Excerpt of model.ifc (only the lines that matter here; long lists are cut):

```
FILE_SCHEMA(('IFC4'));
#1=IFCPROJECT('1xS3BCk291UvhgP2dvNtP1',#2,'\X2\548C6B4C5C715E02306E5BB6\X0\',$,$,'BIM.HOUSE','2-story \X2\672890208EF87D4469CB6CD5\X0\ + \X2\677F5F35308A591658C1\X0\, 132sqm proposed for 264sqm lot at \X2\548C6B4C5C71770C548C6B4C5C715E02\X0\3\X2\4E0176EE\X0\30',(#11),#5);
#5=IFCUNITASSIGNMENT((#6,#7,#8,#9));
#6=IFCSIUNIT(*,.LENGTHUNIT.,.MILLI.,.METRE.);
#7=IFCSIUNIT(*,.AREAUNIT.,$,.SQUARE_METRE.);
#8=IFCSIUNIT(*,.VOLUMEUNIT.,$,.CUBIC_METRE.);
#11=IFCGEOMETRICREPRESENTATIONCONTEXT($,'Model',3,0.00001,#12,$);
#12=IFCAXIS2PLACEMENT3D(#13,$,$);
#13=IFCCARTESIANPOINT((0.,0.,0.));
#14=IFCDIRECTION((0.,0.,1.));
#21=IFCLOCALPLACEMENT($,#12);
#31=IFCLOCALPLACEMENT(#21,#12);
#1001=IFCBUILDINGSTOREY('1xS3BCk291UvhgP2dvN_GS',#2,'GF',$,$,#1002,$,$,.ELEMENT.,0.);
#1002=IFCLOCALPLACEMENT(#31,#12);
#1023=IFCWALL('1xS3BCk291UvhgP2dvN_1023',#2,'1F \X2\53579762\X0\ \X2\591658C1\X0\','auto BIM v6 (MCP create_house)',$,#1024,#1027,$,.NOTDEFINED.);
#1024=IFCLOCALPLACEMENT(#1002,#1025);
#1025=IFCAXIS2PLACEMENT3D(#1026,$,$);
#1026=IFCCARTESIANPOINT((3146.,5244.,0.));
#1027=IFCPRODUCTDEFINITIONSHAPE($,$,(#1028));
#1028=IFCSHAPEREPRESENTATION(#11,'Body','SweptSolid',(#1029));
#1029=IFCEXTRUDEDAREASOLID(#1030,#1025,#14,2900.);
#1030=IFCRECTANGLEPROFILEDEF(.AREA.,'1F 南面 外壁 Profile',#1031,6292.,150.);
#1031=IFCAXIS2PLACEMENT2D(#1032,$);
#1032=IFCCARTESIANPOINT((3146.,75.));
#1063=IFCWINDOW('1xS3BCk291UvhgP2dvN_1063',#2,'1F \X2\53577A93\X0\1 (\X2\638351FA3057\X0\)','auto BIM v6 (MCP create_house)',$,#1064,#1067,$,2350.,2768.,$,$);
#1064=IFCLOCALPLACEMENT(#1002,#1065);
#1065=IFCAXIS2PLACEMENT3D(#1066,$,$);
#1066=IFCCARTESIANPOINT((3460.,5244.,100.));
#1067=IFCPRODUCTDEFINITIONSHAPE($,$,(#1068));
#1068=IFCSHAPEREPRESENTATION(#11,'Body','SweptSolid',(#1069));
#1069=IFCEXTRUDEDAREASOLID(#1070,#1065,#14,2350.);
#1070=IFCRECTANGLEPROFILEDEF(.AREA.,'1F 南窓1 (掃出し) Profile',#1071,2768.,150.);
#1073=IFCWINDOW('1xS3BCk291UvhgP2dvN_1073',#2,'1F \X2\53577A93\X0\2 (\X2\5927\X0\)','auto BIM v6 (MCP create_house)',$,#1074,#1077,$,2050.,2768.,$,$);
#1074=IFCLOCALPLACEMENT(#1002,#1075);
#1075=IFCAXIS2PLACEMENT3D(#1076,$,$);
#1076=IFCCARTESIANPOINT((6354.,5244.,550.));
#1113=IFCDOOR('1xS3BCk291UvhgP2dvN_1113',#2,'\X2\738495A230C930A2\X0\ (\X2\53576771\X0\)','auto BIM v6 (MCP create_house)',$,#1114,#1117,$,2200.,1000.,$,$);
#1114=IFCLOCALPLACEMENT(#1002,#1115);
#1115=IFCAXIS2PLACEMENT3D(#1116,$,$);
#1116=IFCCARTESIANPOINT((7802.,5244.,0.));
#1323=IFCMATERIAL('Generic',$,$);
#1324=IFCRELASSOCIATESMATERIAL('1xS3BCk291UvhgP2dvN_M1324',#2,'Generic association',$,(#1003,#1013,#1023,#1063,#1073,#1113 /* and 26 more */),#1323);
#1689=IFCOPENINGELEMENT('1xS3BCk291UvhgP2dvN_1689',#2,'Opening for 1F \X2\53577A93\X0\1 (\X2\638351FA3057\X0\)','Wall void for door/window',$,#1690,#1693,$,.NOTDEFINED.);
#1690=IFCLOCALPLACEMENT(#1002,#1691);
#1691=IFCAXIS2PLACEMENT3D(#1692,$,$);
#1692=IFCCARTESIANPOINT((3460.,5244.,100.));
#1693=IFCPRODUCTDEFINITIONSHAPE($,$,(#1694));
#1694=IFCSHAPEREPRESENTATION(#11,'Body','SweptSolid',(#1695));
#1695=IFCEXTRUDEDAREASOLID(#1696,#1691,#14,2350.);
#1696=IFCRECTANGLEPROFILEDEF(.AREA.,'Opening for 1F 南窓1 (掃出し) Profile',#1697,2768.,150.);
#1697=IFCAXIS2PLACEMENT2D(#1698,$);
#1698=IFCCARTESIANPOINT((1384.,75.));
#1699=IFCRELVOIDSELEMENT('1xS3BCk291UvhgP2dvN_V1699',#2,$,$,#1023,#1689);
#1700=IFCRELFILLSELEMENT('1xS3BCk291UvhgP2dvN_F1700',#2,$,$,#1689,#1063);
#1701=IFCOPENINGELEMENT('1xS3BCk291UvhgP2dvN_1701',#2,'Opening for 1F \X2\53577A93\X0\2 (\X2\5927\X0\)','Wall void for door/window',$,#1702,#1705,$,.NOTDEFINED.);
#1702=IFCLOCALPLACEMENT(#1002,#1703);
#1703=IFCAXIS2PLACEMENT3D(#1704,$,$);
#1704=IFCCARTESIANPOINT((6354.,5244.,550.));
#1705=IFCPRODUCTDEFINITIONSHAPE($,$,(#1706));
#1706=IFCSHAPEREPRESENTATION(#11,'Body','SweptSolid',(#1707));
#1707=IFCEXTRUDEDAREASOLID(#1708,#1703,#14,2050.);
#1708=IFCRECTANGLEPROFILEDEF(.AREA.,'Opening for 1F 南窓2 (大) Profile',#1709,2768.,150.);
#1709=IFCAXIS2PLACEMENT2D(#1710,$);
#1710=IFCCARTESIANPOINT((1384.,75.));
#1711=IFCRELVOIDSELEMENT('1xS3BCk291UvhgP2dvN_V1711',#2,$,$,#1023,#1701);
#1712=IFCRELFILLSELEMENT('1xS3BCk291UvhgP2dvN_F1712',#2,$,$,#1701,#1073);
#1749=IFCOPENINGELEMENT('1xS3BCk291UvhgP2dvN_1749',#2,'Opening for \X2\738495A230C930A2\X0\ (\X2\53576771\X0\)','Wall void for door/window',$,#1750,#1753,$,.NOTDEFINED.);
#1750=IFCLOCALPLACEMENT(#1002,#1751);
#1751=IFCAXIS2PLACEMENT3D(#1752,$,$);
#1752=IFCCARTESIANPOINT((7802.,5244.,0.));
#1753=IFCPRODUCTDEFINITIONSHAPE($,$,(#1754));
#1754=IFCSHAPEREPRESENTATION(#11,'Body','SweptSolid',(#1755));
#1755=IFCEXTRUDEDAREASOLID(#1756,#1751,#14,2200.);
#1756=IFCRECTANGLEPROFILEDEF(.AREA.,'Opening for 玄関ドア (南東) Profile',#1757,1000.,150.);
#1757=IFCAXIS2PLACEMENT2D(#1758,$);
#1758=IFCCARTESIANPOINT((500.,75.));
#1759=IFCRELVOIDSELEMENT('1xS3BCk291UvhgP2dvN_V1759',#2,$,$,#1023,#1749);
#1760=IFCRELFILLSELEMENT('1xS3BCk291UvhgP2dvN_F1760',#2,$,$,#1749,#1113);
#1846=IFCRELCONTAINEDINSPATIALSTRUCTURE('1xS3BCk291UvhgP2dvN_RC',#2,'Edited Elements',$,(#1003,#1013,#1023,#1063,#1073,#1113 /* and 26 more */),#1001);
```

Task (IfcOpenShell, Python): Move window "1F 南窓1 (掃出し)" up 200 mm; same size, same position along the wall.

```python
import numpy as np
import ifcopenshell
import ifcopenshell.api.geometry
import ifcopenshell.util.placement
import ifcopenshell.util.unit

model = ifcopenshell.open("model.ifc")
unit_scale = ifcopenshell.util.unit.calculate_unit_scale(model)

window = model.by_guid("1xS3BCk291UvhgP2dvN_1063")
opening = window.FillsVoids[0].RelatingOpeningElement
dz = 0.2 / unit_scale

shift = np.array([0.0, 0.0, dz])
# The window is not placed relative to its opening, so move both.
for product in (opening, window):
    matrix = ifcopenshell.util.placement.get_local_placement(product.ObjectPlacement)
    matrix[:3, 3] += shift
    ifcopenshell.api.geometry.edit_object_placement(model, product=product, matrix=matrix, is_si=False)

print(f"moved by {dz * unit_scale:+.3f} m")

model.write("model_edited.ifc")
```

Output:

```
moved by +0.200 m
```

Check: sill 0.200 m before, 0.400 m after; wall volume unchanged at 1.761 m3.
